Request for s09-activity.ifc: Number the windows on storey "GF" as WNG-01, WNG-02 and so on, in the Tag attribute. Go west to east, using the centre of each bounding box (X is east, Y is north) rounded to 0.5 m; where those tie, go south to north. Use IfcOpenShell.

First a look at what the model holds.

```python
import ifcopenshell
import ifcopenshell.util.element
import ifcopenshell.util.placement

model = ifcopenshell.open("s09-activity.ifc")
print(model.schema)
storey = next(s for s in model.by_type("IfcBuildingStorey") if s.Name == "GF")
windows = [e for e in ifcopenshell.util.element.get_decomposition(storey) if e.is_a("IfcWindow")]
for e in sorted(windows, key=lambda e: e.id()):
    origin = ifcopenshell.util.placement.get_local_placement(e.ObjectPlacement)[:3, 3]
    print(e.id(), e.Tag, e.Name, origin.round(2) + 0.0, sep=" | ")
```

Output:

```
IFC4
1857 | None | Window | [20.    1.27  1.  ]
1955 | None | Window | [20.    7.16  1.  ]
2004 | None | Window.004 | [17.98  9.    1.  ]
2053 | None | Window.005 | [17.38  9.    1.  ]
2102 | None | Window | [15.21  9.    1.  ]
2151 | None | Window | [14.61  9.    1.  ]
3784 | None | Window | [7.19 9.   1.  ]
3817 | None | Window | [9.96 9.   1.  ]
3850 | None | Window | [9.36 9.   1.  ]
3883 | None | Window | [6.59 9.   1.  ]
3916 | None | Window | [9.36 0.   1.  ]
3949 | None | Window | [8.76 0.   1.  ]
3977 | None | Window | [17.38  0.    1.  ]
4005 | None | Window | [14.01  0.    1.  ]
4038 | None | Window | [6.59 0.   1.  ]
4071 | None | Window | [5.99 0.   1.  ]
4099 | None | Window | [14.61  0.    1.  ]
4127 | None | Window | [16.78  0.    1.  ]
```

```python
import ifcopenshell
import ifcopenshell.geom
import ifcopenshell.util.element
import ifcopenshell.util.shape

model = ifcopenshell.open("s09-activity.ifc")
settings = ifcopenshell.geom.settings()
settings.set("use-world-coords", True)


def centre(element):
    shape = ifcopenshell.geom.create_shape(settings, element)
    return ifcopenshell.util.shape.get_bbox_centroid(shape.geometry)


storey = next(s for s in model.by_type("IfcBuildingStorey") if s.Name == "GF")
windows = [e for e in ifcopenshell.util.element.get_decomposition(storey) if e.is_a("IfcWindow")]

# Insertion points can sit at a corner or the storey origin, so sort by the geometry (in metres).
centres = {e: centre(e) for e in windows}
windows.sort(key=lambda e: (round(centres[e][0] / 0.5), centres[e][1]))

for i, e in enumerate(windows, start=1):
    number = f"WNG-{i:02d}"
    e.Tag = number
    print(e.id(), number)

model.write("s09-activity_edited.ifc")
```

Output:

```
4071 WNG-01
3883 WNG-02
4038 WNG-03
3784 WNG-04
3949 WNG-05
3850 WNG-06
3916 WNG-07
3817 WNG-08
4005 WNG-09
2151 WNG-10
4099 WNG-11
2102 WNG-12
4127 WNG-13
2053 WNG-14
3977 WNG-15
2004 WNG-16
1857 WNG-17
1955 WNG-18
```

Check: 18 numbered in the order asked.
